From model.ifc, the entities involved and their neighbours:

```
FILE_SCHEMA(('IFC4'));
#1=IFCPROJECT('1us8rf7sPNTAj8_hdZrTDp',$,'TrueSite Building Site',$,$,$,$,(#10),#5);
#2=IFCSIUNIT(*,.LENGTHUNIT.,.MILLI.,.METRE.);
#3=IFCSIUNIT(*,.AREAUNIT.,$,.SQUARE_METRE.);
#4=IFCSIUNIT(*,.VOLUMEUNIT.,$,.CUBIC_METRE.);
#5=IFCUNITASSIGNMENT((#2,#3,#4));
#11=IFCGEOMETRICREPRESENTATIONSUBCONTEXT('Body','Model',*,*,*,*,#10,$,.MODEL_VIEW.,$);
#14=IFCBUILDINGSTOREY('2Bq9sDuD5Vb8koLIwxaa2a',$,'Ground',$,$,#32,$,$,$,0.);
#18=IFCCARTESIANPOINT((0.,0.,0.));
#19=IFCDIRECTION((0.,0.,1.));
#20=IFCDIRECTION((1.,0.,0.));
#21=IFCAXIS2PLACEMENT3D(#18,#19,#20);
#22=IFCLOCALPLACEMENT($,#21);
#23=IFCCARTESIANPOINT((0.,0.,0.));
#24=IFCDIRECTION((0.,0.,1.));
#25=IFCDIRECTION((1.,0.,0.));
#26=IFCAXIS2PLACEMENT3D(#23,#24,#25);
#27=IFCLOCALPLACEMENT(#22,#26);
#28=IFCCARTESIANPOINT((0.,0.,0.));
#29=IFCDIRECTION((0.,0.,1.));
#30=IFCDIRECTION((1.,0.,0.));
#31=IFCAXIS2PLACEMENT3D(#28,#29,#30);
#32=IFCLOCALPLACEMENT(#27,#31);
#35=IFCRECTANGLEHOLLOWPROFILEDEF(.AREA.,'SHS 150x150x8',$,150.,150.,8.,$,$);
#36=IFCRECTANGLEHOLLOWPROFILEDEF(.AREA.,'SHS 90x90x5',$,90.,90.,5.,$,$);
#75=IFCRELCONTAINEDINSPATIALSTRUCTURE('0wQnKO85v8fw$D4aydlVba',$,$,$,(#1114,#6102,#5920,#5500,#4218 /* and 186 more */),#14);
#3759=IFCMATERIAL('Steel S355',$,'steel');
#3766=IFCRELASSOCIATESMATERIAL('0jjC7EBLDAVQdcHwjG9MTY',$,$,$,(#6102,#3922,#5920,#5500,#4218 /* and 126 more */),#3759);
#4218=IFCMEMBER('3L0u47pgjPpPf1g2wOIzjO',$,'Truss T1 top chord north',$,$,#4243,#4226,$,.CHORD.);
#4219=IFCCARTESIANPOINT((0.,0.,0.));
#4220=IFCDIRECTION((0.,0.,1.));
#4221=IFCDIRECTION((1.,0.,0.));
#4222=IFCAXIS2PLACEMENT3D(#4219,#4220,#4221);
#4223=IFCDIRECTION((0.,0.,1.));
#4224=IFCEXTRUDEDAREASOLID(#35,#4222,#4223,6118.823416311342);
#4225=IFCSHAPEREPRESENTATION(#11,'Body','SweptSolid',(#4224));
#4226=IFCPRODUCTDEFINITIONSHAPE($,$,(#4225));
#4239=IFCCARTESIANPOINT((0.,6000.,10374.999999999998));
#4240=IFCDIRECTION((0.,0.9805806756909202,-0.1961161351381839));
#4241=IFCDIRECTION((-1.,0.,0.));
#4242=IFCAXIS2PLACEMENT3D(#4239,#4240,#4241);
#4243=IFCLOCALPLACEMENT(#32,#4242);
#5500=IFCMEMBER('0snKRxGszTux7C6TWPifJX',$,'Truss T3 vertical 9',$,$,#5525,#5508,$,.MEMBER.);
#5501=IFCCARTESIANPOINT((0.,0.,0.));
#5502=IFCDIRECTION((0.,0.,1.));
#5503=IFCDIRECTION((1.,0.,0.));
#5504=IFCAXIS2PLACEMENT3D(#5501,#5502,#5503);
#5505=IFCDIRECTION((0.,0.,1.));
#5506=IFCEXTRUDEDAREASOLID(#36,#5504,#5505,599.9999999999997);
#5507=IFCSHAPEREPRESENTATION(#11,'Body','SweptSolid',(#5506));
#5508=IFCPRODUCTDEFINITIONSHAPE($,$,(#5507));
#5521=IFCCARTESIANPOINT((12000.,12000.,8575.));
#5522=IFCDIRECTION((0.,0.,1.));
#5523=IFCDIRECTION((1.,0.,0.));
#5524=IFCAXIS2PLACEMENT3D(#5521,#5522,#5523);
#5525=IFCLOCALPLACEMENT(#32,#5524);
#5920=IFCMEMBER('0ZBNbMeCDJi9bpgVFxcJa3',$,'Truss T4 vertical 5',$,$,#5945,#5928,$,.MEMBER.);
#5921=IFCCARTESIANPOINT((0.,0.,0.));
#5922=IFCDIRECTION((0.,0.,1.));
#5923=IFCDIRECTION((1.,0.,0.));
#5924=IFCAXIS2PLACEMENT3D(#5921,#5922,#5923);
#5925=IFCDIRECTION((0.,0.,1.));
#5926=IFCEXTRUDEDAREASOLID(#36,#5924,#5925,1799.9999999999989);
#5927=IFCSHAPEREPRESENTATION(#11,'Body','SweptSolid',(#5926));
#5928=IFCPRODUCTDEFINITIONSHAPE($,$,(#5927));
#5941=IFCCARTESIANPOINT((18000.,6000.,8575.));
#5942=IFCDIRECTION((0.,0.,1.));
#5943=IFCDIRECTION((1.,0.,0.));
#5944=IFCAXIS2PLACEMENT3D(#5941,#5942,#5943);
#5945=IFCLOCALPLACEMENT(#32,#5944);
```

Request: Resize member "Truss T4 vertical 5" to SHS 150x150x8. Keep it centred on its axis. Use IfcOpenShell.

```python
import ifcopenshell
import ifcopenshell.util.element
import ifcopenshell.util.representation

model = ifcopenshell.open("model.ifc")

member = model.by_guid("0ZBNbMeCDJi9bpgVFxcJa3")
source = next(p for p in model.by_type("IfcRectangleHollowProfileDef") if p.ProfileName == "SHS 150x150x8")

body = ifcopenshell.util.representation.get_representation(member, "Model", "Body")
solid = body.Items[0]
old_profile = solid.SweptArea

# Copy the section's sizes but keep this member's own profile position.
profile = ifcopenshell.util.element.copy(model, source)
profile.Position = old_profile.Position
solid.SweptArea = profile
if not model.get_total_inverses(old_profile):
    ifcopenshell.util.element.remove_deep2(model, old_profile)

print(solid.SweptArea)

model.write("model_v2.ifc")
```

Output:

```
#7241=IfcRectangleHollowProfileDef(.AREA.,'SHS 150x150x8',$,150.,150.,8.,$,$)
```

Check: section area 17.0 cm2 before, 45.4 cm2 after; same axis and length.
